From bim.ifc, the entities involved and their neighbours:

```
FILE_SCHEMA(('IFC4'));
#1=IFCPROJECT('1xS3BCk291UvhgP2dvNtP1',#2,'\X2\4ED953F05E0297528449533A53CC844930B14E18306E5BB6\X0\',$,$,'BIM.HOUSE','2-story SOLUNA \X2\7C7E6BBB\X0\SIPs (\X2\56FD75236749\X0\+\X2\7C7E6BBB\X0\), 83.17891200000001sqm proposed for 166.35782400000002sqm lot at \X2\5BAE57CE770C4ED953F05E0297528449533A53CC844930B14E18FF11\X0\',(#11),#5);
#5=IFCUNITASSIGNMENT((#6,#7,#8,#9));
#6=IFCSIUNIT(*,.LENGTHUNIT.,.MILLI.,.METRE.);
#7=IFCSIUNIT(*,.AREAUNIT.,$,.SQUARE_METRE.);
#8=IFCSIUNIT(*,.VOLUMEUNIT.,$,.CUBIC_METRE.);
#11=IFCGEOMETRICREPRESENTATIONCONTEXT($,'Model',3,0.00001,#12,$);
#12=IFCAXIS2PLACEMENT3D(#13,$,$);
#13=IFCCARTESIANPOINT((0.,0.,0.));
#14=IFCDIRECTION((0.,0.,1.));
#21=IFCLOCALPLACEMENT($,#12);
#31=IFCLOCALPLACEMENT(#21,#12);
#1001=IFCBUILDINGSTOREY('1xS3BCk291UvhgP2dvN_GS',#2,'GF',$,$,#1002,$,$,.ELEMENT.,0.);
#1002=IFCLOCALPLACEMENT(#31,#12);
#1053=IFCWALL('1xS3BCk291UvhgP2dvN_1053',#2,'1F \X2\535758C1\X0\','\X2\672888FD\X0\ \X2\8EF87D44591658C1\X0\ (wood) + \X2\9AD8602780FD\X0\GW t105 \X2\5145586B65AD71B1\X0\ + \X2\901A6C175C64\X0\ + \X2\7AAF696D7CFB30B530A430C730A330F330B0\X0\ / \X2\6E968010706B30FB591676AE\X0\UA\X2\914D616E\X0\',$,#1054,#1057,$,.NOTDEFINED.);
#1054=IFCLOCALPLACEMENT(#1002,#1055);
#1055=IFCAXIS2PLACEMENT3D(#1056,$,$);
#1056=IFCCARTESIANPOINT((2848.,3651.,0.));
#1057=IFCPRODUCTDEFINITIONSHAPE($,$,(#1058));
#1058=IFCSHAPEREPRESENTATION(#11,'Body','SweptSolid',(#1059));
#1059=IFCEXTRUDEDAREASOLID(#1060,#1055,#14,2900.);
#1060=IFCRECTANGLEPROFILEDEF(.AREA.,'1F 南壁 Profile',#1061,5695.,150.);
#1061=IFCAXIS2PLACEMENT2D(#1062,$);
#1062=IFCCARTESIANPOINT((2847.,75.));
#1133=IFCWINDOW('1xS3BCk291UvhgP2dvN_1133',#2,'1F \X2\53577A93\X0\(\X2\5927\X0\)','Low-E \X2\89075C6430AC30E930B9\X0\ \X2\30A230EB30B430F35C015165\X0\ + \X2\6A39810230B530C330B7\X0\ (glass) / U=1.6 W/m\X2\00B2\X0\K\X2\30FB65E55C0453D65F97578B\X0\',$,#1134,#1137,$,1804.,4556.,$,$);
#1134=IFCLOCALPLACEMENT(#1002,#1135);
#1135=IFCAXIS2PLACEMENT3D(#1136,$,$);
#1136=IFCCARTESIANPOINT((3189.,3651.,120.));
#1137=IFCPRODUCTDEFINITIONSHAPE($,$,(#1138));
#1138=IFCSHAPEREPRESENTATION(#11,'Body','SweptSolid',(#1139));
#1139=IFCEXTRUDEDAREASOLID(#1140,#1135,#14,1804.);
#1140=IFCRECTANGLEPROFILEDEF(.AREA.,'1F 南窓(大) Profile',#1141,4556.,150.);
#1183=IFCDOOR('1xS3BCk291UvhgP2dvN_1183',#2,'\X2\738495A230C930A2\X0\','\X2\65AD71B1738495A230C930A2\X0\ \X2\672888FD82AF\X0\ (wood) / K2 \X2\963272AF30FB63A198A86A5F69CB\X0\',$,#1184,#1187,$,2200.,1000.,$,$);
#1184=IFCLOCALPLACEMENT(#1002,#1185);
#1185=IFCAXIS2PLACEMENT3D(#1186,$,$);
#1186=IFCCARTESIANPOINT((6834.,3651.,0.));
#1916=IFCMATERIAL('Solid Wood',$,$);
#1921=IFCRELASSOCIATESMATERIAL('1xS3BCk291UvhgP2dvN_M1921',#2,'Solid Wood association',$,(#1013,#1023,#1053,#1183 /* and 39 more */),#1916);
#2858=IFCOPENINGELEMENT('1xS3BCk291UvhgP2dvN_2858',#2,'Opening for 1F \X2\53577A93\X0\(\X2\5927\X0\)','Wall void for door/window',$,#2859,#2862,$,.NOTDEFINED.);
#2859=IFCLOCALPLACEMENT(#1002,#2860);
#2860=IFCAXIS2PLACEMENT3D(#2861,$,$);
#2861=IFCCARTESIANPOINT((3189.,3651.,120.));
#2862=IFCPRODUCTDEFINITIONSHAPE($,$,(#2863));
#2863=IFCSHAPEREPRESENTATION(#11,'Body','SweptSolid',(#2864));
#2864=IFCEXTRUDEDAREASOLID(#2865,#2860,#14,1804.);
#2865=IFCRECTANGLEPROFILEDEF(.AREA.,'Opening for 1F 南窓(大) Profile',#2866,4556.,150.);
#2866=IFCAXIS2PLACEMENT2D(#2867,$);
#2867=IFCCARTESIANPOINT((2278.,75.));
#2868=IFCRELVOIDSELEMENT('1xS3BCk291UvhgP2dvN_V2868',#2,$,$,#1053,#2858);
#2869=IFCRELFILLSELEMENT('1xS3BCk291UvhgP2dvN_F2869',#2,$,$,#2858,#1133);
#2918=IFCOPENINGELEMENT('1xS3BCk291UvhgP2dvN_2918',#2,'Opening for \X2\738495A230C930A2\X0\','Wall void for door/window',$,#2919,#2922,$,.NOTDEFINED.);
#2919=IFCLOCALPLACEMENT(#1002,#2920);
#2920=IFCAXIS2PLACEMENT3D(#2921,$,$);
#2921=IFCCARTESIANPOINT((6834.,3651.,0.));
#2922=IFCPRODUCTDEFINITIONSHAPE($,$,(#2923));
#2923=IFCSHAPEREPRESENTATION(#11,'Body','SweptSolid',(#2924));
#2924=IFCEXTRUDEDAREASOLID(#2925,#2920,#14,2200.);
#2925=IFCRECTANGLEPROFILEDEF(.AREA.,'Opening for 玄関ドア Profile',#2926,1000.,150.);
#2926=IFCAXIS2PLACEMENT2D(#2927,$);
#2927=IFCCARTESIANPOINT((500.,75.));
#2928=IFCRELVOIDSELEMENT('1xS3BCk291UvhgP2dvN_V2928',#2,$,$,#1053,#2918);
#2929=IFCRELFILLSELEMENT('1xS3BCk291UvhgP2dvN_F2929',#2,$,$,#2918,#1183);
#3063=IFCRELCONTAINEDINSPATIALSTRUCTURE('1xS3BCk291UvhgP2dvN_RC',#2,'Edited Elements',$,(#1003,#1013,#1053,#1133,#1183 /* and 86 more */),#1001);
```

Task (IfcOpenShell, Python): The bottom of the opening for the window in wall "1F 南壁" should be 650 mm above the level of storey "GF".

```python
import numpy as np
import ifcopenshell
import ifcopenshell.api.geometry
import ifcopenshell.geom
import ifcopenshell.util.element
import ifcopenshell.util.placement
import ifcopenshell.util.shape
import ifcopenshell.util.unit

model = ifcopenshell.open("bim.ifc")
unit_scale = ifcopenshell.util.unit.calculate_unit_scale(model)

window = model.by_guid("1xS3BCk291UvhgP2dvN_1133")
opening = window.FillsVoids[0].RelatingOpeningElement
storey = ifcopenshell.util.element.get_container(window, ifc_class="IfcBuildingStorey")
level = ifcopenshell.util.placement.get_local_placement(storey.ObjectPlacement)[2, 3]

# The opening's origin need not be at the sill, so measure its lowest point.
shape = ifcopenshell.geom.create_shape(ifcopenshell.geom.settings(), opening)
bottom = ifcopenshell.util.shape.get_shape_bottom_elevation(shape, shape.geometry) / unit_scale
dz = level + 650.0 - bottom

shift = np.array([0.0, 0.0, dz])
# The window is not placed relative to its opening, so move both.
for product in (opening, window):
    matrix = ifcopenshell.util.placement.get_local_placement(product.ObjectPlacement)
    matrix[:3, 3] += shift
    ifcopenshell.api.geometry.edit_object_placement(model, product=product, matrix=matrix, is_si=False)

print(f"moved by {dz * unit_scale:+.3f} m")

model.write("bim_edited.ifc")
```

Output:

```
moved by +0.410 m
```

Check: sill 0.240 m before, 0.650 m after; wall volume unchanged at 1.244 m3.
